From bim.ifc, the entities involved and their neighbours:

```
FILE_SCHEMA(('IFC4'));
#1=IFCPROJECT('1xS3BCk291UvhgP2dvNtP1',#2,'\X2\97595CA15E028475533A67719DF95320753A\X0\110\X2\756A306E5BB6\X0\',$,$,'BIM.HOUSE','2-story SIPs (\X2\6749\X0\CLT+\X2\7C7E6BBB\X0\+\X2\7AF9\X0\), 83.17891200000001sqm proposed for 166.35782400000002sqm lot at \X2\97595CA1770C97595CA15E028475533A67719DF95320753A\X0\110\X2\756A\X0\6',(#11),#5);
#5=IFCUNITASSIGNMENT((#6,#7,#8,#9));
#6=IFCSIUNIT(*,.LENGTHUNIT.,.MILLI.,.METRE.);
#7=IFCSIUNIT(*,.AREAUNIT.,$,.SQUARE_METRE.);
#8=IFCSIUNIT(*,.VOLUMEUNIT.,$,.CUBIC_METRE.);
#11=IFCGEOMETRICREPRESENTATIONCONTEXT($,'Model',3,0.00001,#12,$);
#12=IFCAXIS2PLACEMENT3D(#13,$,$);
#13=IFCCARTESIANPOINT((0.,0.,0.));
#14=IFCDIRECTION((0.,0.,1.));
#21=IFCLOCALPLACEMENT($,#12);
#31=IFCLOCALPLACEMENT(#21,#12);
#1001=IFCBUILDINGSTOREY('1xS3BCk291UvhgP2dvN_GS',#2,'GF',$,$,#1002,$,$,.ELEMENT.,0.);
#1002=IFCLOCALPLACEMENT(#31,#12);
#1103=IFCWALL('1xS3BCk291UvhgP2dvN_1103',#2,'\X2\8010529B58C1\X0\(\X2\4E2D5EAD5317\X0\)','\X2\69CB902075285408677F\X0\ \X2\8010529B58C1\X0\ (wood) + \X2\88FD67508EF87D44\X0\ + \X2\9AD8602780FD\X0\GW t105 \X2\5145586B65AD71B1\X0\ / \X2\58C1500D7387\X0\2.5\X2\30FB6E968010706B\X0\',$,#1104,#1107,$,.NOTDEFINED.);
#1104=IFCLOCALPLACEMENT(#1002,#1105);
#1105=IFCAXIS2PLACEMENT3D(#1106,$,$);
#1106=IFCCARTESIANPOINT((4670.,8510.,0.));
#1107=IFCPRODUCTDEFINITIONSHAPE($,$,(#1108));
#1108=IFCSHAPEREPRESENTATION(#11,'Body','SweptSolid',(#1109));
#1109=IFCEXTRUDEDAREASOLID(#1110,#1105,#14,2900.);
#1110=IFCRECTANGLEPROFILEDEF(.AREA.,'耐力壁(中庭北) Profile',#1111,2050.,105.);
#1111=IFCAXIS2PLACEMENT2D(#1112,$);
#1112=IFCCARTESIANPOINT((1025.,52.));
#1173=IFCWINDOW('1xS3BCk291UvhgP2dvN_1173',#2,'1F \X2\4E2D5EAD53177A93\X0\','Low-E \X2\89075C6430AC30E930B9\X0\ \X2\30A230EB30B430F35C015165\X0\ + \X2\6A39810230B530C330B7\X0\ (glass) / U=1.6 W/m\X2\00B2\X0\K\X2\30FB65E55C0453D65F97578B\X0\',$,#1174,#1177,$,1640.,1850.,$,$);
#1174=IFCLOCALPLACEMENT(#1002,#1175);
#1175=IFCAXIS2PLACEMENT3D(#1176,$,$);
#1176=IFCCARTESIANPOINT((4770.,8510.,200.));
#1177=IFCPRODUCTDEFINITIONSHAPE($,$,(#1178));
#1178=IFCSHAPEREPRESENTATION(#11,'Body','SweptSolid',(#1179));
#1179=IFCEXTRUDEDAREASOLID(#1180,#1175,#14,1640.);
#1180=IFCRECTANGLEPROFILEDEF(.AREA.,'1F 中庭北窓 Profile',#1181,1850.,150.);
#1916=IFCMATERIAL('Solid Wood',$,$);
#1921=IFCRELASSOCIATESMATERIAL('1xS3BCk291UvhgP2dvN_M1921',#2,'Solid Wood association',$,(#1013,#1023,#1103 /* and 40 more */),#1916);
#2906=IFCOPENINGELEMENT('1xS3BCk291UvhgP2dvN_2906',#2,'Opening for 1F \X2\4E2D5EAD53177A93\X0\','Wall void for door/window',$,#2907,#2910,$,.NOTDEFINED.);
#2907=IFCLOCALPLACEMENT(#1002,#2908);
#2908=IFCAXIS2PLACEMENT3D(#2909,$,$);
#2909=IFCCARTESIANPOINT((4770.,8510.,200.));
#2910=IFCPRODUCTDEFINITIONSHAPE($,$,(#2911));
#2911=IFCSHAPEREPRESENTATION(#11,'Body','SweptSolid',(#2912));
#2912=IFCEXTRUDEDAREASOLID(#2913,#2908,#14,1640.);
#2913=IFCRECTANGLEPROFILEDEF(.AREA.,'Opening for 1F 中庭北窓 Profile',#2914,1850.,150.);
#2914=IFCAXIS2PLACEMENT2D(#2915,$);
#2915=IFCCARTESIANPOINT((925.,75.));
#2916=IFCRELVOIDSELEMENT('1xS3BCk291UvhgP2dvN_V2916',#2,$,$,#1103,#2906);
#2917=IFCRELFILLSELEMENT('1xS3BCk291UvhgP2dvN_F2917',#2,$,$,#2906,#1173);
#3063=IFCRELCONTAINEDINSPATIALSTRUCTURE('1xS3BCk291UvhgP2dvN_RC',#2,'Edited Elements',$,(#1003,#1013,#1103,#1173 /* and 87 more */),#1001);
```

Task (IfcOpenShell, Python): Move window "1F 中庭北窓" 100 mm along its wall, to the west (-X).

```python
import ifcopenshell
import ifcopenshell.api.geometry
import ifcopenshell.util.placement
import ifcopenshell.util.unit

model = ifcopenshell.open("bim.ifc")
unit_scale = ifcopenshell.util.unit.calculate_unit_scale(model)

window = model.by_id(1173)
opening = window.FillsVoids[0].RelatingOpeningElement
wall = opening.VoidsElements[0].RelatingBuildingElement

wall_matrix = ifcopenshell.util.placement.get_local_placement(wall.ObjectPlacement)
shift = wall_matrix[:3, 0] * -0.1 / unit_scale
before = ifcopenshell.util.placement.get_local_placement(window.ObjectPlacement)[:3, 3].copy()

# The window is not placed relative to its opening, so move both.
for product in (opening, window):
    matrix = ifcopenshell.util.placement.get_local_placement(product.ObjectPlacement)
    matrix[:3, 3] += shift
    ifcopenshell.api.geometry.edit_object_placement(model, product=product, matrix=matrix, is_si=False)

after = ifcopenshell.util.placement.get_local_placement(window.ObjectPlacement)[:3, 3]
print("window moved by", (after - before).round(3) + 0.0)

model.write("bim_v2.ifc")
```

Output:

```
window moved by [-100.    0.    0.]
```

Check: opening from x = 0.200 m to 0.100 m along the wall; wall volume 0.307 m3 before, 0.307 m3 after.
